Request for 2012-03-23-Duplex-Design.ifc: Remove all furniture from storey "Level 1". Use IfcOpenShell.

First a look at what the model holds.

```python
import ifcopenshell
import ifcopenshell.util.element

model = ifcopenshell.open("2012-03-23-Duplex-Design.ifc")
print(model.schema)
storey = next(s for s in model.by_type("IfcBuildingStorey") if s.Name == "Level 1")
furniture = [e for e in ifcopenshell.util.element.get_decomposition(storey) if e.is_a("IfcFurnishingElement")]
seen = {}
for e in furniture:
    element_type = ifcopenshell.util.element.get_type(e)
    name = element_type.Name if element_type not in (None, e) else None
    seen[name] = seen.get(name, 0) + 1
for name, count in sorted(seen.items(), key=str):
    print(count, "x", name)
```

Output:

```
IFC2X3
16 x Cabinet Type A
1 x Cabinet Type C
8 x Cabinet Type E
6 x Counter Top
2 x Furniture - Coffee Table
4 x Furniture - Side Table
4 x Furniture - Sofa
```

```python
import ifcopenshell
import ifcopenshell.api.root
import ifcopenshell.util.element

model = ifcopenshell.open("2012-03-23-Duplex-Design.ifc")

storey = next(s for s in model.by_type("IfcBuildingStorey") if s.Name == "Level 1")
furniture = [e for e in ifcopenshell.util.element.get_decomposition(storey) if e.is_a("IfcFurnishingElement")]

for e in furniture:
    ifcopenshell.api.root.remove_product(model, product=e)
print(len(furniture), "removed")

model.write("2012-03-23-Duplex-Design_edited.ifc")
```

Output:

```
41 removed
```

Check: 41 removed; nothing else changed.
